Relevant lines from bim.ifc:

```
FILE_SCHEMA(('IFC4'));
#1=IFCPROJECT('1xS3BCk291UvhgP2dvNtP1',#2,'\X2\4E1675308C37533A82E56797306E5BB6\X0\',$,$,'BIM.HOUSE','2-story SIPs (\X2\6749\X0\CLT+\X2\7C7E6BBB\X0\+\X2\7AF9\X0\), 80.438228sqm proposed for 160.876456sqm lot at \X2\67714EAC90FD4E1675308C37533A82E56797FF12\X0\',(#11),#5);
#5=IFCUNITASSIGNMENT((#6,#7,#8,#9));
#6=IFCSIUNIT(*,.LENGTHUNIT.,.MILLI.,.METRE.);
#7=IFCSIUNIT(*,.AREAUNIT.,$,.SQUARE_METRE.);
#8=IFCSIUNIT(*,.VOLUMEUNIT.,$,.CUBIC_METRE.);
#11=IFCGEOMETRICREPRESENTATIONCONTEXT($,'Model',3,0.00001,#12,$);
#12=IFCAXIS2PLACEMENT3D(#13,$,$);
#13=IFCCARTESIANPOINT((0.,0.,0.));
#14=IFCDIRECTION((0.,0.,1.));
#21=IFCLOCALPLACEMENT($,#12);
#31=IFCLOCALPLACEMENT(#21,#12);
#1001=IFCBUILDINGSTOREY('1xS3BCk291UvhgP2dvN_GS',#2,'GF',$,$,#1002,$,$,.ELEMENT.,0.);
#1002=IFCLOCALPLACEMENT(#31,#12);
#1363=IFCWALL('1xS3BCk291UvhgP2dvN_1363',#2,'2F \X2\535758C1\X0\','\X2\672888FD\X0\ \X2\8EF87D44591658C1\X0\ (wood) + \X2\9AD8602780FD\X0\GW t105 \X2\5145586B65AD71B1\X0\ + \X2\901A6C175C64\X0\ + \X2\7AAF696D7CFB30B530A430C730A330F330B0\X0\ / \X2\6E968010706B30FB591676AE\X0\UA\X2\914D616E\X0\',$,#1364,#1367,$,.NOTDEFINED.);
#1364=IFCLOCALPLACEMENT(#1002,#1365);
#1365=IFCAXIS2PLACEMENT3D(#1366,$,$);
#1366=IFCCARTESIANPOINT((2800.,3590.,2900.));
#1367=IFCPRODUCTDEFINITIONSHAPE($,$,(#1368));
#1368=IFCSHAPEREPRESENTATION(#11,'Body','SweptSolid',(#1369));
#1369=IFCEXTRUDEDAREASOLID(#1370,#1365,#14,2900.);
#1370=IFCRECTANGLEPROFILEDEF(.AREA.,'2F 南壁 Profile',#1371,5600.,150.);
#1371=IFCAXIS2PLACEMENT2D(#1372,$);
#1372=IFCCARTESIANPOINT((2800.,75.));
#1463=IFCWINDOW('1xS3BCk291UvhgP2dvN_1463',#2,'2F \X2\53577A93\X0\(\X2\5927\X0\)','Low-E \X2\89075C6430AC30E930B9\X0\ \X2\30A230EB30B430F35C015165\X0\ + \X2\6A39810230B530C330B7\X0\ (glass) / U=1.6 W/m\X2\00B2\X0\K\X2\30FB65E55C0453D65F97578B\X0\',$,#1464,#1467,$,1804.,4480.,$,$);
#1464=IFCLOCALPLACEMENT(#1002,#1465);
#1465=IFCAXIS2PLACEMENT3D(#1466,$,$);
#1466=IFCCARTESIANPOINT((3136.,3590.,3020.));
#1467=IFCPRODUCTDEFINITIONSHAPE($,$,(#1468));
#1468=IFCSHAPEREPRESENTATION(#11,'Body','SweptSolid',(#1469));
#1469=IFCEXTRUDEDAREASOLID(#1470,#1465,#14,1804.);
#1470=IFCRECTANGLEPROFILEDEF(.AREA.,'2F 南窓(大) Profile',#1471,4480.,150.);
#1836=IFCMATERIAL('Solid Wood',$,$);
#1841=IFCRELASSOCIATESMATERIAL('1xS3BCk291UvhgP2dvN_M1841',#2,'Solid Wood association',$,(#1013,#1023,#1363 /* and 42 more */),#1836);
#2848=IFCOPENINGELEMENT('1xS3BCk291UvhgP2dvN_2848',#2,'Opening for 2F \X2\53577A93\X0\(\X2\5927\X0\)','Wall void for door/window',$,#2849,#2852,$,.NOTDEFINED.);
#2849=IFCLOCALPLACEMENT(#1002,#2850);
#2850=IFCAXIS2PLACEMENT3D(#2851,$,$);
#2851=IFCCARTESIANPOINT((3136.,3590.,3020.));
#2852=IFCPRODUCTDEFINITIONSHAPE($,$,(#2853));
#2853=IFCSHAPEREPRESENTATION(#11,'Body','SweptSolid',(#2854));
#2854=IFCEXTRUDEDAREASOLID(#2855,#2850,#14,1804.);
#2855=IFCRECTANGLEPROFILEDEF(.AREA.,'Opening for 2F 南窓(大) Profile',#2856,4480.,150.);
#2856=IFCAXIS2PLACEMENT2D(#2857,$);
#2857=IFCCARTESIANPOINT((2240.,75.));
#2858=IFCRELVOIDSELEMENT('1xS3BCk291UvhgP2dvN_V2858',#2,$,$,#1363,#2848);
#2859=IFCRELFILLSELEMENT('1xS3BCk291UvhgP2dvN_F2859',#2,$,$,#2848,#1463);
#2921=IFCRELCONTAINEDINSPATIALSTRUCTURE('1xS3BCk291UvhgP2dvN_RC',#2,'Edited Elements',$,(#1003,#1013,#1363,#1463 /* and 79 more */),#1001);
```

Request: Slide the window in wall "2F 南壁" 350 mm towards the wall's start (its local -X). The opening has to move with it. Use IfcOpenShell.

```python
import ifcopenshell
import ifcopenshell.api.geometry
import ifcopenshell.util.placement

model = ifcopenshell.open("bim.ifc")

window = model.by_guid("1xS3BCk291UvhgP2dvN_1463")
opening = window.FillsVoids[0].RelatingOpeningElement
wall = opening.VoidsElements[0].RelatingBuildingElement

wall_matrix = ifcopenshell.util.placement.get_local_placement(wall.ObjectPlacement)
shift = wall_matrix[:3, 0] * -350.0
before = ifcopenshell.util.placement.get_local_placement(window.ObjectPlacement)[:3, 3].copy()

# The window is not placed relative to its opening, so move both.
for product in (opening, window):
    matrix = ifcopenshell.util.placement.get_local_placement(product.ObjectPlacement)
    matrix[:3, 3] += shift
    ifcopenshell.api.geometry.edit_object_placement(model, product=product, matrix=matrix, is_si=False)

after = ifcopenshell.util.placement.get_local_placement(window.ObjectPlacement)[:3, 3]
print("window moved by", (after - before).round(3) + 0.0)

model.write("bim-out.ifc")
```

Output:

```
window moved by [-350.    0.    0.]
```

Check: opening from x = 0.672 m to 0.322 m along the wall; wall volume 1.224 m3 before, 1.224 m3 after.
